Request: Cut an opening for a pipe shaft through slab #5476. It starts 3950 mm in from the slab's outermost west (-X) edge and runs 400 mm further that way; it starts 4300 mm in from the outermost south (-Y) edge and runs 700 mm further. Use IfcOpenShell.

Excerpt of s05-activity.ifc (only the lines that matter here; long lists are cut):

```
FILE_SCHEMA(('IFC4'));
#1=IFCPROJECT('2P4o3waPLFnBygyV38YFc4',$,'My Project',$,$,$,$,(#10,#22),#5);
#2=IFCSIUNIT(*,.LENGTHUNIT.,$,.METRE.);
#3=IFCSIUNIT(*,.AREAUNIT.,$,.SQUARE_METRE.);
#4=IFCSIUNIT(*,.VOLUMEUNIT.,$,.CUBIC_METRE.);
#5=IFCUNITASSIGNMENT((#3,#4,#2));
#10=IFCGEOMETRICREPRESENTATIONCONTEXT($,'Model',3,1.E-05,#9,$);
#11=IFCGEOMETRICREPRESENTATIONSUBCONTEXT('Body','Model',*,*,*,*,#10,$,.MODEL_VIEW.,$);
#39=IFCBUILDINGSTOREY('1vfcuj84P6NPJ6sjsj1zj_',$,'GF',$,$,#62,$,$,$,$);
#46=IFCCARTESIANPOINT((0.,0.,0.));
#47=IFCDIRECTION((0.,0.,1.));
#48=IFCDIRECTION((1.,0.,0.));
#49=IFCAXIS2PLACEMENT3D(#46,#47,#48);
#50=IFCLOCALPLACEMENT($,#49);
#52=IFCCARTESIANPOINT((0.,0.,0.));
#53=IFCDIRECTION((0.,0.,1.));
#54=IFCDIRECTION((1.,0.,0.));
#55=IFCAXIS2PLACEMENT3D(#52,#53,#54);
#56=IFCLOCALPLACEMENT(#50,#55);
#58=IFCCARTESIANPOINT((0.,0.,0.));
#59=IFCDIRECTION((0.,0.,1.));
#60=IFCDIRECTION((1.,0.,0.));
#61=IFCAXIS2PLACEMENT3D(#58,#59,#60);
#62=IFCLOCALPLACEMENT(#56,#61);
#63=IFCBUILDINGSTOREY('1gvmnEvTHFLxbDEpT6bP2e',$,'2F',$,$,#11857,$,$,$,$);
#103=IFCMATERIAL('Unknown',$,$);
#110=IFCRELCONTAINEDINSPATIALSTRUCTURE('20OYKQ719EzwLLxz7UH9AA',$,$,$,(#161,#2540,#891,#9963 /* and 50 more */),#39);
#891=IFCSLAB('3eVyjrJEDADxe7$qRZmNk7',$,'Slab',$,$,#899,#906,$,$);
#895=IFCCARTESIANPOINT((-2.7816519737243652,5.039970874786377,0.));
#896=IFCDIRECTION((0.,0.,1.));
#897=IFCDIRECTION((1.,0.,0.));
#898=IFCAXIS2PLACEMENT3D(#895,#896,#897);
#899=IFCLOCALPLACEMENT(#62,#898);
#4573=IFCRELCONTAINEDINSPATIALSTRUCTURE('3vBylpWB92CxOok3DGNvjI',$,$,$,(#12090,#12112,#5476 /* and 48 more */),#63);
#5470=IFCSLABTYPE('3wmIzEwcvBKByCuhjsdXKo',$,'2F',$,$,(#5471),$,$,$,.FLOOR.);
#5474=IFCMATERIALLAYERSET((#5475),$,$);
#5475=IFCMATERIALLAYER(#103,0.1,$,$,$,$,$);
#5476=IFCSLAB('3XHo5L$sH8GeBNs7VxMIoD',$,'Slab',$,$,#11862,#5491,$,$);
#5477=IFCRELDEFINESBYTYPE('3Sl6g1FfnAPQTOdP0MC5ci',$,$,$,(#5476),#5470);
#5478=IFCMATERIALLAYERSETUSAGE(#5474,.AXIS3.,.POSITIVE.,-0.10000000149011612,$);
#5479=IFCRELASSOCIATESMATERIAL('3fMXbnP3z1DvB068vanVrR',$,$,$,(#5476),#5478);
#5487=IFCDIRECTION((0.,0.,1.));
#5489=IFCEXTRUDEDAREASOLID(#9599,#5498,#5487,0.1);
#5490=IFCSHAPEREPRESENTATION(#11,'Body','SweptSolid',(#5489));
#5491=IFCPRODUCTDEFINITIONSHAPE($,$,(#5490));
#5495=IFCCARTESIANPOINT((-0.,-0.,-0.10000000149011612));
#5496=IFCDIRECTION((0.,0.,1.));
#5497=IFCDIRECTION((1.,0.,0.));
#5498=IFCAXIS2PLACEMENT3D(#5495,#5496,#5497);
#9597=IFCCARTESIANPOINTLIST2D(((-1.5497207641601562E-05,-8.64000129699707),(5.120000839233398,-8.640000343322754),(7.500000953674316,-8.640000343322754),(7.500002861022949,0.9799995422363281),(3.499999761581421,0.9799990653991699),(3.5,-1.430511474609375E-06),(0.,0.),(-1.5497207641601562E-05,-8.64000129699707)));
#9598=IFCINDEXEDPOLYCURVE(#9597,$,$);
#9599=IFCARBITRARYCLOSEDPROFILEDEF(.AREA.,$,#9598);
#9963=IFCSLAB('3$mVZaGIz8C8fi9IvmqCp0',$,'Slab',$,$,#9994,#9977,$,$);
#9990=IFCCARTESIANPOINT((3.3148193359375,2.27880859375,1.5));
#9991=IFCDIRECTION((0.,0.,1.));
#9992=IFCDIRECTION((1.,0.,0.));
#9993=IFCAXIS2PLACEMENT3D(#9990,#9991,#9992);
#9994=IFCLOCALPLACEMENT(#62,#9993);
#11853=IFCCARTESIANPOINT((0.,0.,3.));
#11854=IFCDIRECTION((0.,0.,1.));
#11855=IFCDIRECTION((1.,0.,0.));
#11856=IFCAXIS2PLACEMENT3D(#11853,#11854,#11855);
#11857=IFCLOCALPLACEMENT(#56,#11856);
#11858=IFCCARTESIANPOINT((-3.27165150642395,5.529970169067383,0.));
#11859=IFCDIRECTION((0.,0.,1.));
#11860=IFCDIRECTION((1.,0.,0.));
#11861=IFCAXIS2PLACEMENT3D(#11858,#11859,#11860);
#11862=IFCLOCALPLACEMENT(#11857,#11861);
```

```python
import numpy as np
import ifcopenshell
import ifcopenshell.api.feature
import ifcopenshell.api.geometry
import ifcopenshell.api.root
import ifcopenshell.geom
import ifcopenshell.util.placement
import ifcopenshell.util.representation
import ifcopenshell.util.shape
import ifcopenshell.util.unit

model = ifcopenshell.open("s05-activity.ifc")
unit_scale = ifcopenshell.util.unit.calculate_unit_scale(model)
settings = ifcopenshell.geom.settings()


def volume(element):
    """Net volume in cubic metres, openings subtracted."""
    shape = ifcopenshell.geom.create_shape(settings, element)
    return ifcopenshell.util.shape.get_volume(shape.geometry)


slab = model.by_guid("3XHo5L$sH8GeBNs7VxMIoD")
before = volume(slab)

# Extent in the slab's own axes, in metres. The edges named are its -X and -Y sides.
slab_shape = ifcopenshell.geom.create_shape(settings, slab)
vertices = ifcopenshell.util.shape.get_vertices(slab_shape.geometry)
x_min, y_min, bottom = vertices.min(axis=0)
top = vertices[:, 2].max()

opening = ifcopenshell.api.root.create_entity(model, ifc_class="IfcOpeningElement", name="Pipe shaft opening", predefined_type="OPENING")
context = ifcopenshell.util.representation.get_context(model, "Model", "Body", "MODEL_VIEW")
width, depth = 0.4, 0.7
outline = [(0.0, 0.0), (width, 0.0), (width, depth), (0.0, depth), (0.0, 0.0)]
# Overshoot both faces by 50 mm so the cut is clean.
shape = ifcopenshell.api.geometry.add_slab_representation(
    model, context=context, depth=top - bottom + 0.1, polyline=outline
)
ifcopenshell.api.geometry.assign_representation(model, product=opening, representation=shape)

matrix = ifcopenshell.util.placement.get_local_placement(slab.ObjectPlacement)
matrix[:, 3] = matrix @ np.append(np.array([x_min + 3.95, y_min + 4.3, bottom - 0.05]) / unit_scale, 1.0)
ifcopenshell.api.geometry.edit_object_placement(model, product=opening, matrix=matrix, is_si=False)
ifcopenshell.api.feature.add_feature(model, feature=opening, element=slab)

after = volume(slab)

print(f"slab volume {before:.3f} -> {after:.3f} m3")

model.write("s05-activity_updated.ifc")
```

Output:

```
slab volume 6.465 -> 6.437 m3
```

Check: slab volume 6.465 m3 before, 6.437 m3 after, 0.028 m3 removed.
